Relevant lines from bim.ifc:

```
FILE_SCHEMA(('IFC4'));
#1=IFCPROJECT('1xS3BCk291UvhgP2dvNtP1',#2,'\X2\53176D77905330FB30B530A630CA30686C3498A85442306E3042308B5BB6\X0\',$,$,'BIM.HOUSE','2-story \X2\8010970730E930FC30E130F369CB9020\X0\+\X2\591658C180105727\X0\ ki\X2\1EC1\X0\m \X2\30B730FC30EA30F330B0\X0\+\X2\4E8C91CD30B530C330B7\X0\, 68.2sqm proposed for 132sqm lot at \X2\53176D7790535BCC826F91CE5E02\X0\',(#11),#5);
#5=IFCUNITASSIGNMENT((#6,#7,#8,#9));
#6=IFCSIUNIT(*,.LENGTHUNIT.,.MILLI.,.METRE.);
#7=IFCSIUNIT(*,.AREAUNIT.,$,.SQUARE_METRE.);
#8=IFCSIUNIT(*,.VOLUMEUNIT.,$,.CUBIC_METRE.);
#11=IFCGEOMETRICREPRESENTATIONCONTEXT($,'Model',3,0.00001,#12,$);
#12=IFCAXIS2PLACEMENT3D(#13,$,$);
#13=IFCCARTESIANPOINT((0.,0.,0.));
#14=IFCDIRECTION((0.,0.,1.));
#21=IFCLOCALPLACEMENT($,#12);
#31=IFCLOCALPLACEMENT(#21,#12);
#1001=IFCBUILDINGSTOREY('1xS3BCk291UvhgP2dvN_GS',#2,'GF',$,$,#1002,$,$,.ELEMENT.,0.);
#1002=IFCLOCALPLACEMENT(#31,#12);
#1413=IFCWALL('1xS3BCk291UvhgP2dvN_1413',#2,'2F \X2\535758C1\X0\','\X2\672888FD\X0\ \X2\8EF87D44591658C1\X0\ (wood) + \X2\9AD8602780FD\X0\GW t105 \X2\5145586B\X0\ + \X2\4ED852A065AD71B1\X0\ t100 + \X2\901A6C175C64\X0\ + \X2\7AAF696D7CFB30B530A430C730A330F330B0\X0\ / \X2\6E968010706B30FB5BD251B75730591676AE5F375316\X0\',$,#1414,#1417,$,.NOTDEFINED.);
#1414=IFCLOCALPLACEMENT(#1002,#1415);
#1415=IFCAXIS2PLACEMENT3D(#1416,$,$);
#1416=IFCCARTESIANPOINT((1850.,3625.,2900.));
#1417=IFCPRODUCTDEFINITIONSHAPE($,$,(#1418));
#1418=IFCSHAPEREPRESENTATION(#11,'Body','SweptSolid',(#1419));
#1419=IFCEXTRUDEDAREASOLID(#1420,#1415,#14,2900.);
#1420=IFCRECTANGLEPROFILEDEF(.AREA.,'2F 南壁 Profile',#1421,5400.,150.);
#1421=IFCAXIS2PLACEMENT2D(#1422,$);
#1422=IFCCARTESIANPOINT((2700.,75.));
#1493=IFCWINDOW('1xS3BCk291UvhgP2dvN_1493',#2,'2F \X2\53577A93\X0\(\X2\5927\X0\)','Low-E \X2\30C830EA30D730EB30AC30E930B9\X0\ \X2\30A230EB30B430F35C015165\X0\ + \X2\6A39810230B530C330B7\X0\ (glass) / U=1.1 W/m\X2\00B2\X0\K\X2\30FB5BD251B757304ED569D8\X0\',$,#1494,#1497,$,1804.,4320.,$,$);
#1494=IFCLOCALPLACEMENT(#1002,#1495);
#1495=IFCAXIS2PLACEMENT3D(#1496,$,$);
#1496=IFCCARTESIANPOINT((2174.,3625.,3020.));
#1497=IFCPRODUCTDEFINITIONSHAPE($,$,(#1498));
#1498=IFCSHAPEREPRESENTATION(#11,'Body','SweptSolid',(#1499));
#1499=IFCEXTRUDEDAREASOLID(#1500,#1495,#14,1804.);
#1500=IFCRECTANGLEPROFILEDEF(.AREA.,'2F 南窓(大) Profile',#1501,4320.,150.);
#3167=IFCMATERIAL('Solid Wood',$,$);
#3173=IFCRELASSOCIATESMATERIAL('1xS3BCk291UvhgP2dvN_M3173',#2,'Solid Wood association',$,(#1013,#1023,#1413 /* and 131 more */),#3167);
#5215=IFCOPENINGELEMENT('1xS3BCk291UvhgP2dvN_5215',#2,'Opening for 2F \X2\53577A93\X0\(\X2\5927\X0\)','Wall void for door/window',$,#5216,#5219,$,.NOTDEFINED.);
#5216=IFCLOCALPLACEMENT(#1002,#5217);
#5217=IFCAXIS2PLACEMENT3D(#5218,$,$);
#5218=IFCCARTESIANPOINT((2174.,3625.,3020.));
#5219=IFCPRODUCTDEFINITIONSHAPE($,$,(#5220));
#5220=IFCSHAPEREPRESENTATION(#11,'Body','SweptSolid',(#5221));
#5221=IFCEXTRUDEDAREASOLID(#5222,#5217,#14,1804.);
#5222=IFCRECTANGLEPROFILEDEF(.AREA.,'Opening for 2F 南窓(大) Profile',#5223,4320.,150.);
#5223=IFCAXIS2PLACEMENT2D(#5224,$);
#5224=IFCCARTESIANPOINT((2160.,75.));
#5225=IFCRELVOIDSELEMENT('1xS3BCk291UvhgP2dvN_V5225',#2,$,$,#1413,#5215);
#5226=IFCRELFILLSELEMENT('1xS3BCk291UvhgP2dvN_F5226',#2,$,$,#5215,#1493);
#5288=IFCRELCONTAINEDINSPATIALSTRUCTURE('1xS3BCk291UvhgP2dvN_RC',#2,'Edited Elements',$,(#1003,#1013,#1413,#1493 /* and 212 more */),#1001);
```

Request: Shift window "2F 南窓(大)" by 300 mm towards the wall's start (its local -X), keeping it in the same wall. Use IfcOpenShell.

```python
import ifcopenshell
import ifcopenshell.api.geometry
import ifcopenshell.util.placement

model = ifcopenshell.open("bim.ifc")

window = model.by_id(1493)
opening = window.FillsVoids[0].RelatingOpeningElement
wall = opening.VoidsElements[0].RelatingBuildingElement

wall_matrix = ifcopenshell.util.placement.get_local_placement(wall.ObjectPlacement)
shift = wall_matrix[:3, 0] * -300.0
before = ifcopenshell.util.placement.get_local_placement(window.ObjectPlacement)[:3, 3].copy()

# The window is not placed relative to its opening, so move both.
for product in (opening, window):
    matrix = ifcopenshell.util.placement.get_local_placement(product.ObjectPlacement)
    matrix[:3, 3] += shift
    ifcopenshell.api.geometry.edit_object_placement(model, product=product, matrix=matrix, is_si=False)

after = ifcopenshell.util.placement.get_local_placement(window.ObjectPlacement)[:3, 3]
print("window moved by", (after - before).round(3) + 0.0)

model.write("bim_rev.ifc")
```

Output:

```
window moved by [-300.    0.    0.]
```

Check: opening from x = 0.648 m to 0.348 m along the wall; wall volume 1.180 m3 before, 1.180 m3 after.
